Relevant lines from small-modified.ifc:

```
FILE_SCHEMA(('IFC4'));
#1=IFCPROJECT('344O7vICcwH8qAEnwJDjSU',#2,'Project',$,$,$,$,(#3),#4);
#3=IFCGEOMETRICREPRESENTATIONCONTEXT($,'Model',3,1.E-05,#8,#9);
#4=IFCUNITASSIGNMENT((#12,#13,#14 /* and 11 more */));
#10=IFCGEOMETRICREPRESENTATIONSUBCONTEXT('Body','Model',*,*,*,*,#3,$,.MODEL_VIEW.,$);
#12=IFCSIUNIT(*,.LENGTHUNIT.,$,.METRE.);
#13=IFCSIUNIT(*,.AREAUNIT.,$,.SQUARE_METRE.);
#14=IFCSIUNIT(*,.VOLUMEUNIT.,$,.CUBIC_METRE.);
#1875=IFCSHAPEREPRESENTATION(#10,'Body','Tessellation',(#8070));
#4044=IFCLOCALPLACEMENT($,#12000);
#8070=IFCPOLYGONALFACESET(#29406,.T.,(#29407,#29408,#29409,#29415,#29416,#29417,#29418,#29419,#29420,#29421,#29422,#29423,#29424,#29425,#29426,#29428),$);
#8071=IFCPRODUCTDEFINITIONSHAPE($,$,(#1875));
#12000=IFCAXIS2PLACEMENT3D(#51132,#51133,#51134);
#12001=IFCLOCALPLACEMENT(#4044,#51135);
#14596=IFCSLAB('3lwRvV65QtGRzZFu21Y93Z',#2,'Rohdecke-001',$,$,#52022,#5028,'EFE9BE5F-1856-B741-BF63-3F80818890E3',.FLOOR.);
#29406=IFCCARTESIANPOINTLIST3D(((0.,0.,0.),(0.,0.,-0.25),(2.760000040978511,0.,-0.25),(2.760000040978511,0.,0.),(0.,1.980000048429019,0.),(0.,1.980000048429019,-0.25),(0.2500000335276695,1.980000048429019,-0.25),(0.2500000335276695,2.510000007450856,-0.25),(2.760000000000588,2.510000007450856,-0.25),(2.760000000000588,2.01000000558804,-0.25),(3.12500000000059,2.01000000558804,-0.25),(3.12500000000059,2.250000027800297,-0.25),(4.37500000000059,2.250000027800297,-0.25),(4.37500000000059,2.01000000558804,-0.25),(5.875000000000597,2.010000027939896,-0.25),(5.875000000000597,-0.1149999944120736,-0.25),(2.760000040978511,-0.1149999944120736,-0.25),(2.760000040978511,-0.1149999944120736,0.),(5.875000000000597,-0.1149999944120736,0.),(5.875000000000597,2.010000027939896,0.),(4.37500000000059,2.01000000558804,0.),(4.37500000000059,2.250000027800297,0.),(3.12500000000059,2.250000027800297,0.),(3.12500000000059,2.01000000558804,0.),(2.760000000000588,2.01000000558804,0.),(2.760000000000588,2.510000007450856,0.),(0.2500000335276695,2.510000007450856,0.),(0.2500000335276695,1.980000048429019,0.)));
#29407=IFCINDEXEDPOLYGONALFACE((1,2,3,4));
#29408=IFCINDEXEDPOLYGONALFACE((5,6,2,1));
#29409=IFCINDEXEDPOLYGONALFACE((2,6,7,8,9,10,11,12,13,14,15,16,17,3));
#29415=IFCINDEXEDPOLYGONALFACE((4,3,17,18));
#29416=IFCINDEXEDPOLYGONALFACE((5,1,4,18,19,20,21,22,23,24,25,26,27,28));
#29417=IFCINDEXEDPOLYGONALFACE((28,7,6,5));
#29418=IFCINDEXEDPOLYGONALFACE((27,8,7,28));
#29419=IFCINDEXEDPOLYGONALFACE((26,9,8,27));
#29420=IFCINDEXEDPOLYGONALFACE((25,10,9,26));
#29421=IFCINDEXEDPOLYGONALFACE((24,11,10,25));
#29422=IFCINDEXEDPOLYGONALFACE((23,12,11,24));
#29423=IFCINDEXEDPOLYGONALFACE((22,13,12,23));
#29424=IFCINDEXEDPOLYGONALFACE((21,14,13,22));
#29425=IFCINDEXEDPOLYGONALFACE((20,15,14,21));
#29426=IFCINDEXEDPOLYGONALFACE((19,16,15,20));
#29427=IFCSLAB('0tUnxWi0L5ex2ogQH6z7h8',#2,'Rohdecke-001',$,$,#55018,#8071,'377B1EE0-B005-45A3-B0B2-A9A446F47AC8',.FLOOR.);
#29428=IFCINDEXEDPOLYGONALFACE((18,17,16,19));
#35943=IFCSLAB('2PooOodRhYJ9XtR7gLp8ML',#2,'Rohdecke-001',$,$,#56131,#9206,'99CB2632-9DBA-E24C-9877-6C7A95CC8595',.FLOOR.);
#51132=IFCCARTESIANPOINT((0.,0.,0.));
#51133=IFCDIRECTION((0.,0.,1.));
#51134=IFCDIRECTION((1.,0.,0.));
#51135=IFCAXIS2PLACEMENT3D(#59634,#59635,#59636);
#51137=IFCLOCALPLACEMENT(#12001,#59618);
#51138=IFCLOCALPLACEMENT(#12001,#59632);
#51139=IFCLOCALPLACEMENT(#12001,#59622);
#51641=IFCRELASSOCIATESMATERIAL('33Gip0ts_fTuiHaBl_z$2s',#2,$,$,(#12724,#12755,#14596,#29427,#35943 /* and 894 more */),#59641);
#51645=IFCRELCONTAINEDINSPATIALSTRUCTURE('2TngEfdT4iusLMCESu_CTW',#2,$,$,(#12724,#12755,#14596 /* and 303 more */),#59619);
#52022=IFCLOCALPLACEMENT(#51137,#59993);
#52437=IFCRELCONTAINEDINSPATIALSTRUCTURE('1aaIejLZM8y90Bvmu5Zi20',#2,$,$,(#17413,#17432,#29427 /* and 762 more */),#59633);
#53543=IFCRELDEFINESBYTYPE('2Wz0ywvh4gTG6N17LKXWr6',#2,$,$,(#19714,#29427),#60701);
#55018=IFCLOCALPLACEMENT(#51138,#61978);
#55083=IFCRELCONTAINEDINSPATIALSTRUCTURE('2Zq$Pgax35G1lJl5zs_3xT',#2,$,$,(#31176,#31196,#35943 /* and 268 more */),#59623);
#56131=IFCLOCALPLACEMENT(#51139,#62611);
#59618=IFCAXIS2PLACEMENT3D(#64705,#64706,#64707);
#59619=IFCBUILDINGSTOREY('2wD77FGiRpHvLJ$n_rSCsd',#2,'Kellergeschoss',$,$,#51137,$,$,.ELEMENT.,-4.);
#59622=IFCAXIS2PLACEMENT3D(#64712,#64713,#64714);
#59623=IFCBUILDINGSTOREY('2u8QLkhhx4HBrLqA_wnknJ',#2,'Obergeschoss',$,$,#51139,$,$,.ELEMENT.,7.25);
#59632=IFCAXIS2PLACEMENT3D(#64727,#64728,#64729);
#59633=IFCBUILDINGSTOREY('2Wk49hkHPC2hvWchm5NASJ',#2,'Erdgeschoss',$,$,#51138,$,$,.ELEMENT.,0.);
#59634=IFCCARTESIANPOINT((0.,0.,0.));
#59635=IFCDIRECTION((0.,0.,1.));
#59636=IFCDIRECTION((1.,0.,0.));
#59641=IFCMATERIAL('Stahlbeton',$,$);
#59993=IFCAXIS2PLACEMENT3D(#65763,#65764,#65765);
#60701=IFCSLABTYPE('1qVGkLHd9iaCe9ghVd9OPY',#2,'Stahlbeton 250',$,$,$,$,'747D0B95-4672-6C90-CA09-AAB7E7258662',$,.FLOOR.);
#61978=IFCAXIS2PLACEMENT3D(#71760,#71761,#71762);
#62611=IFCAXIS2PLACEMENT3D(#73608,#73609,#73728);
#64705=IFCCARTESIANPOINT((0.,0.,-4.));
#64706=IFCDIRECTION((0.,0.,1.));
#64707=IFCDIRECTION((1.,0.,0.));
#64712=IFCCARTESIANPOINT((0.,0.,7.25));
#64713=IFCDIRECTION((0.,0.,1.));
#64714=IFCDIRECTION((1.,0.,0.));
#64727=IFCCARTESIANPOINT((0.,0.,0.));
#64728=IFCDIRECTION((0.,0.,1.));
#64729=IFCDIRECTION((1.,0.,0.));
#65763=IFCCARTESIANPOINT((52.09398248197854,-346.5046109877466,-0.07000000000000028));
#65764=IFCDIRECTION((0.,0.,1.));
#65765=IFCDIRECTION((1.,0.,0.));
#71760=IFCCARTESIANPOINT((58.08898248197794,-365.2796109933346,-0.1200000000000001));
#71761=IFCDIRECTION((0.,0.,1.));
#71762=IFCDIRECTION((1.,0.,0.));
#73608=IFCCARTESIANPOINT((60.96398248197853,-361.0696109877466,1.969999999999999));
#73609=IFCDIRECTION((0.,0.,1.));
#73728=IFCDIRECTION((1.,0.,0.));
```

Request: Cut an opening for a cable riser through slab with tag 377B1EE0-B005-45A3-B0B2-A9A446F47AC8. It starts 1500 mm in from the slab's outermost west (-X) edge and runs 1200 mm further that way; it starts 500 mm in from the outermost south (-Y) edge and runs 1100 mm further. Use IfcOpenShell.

```python
import numpy as np
import ifcopenshell
import ifcopenshell.api.feature
import ifcopenshell.api.geometry
import ifcopenshell.api.root
import ifcopenshell.geom
import ifcopenshell.util.placement
import ifcopenshell.util.representation
import ifcopenshell.util.shape
import ifcopenshell.util.unit

model = ifcopenshell.open("small-modified.ifc")
unit_scale = ifcopenshell.util.unit.calculate_unit_scale(model)
settings = ifcopenshell.geom.settings()


def volume(element):
    """Net volume in cubic metres, openings subtracted."""
    shape = ifcopenshell.geom.create_shape(settings, element)
    return ifcopenshell.util.shape.get_volume(shape.geometry)


slab = model.by_id(29427)
before = volume(slab)

# Extent in the slab's own axes, in metres. The edges named are its -X and -Y sides.
slab_shape = ifcopenshell.geom.create_shape(settings, slab)
vertices = ifcopenshell.util.shape.get_vertices(slab_shape.geometry)
x_min, y_min, bottom = vertices.min(axis=0)
top = vertices[:, 2].max()

opening = ifcopenshell.api.root.create_entity(model, ifc_class="IfcOpeningElement", name="Cable riser opening", predefined_type="OPENING")
context = ifcopenshell.util.representation.get_context(model, "Model", "Body", "MODEL_VIEW")
width, depth = 1.2, 1.1
outline = [(0.0, 0.0), (width, 0.0), (width, depth), (0.0, depth), (0.0, 0.0)]
# Overshoot both faces by 50 mm so the cut is clean.
shape = ifcopenshell.api.geometry.add_slab_representation(
    model, context=context, depth=top - bottom + 0.1, polyline=outline
)
ifcopenshell.api.geometry.assign_representation(model, product=opening, representation=shape)

matrix = ifcopenshell.util.placement.get_local_placement(slab.ObjectPlacement)
matrix[:, 3] = matrix @ np.append(np.array([x_min + 1.5, y_min + 0.5, bottom - 0.05]) / unit_scale, 1.0)
ifcopenshell.api.geometry.edit_object_placement(model, product=opening, matrix=matrix, is_si=False)
ifcopenshell.api.feature.add_feature(model, feature=opening, element=slab)

after = volume(slab)

print(f"slab volume {before:.3f} -> {after:.3f} m3")

model.write("small-modified-out.ifc")
```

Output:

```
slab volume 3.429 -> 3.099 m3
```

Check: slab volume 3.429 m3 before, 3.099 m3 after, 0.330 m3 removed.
